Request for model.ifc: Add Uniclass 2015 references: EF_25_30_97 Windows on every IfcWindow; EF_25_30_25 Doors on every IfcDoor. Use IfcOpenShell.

First a look at what the model holds.

```python
import ifcopenshell

model = ifcopenshell.open("model.ifc")
print(model.schema)
print("classifications:", [c.Name for c in model.by_type("IfcClassification")])
for ifc_class in ("IfcDoor", "IfcRoof", "IfcStair", "IfcWall", "IfcWindow"):
    print(ifc_class, len(model.by_type(ifc_class)))
```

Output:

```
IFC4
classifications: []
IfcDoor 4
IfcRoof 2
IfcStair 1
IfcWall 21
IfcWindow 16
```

```python
import ifcopenshell
import ifcopenshell.api.classification

model = ifcopenshell.open("model.ifc")

system = ifcopenshell.api.classification.add_classification(model, classification="Uniclass 2015")

codes = {
    "IfcWindow": ("EF_25_30_97", "Windows"),
    "IfcDoor": ("EF_25_30_25", "Doors"),
}
for ifc_class, (code, name) in codes.items():
    products = model.by_type(ifc_class)
    ifcopenshell.api.classification.add_reference(
        model, products=products, classification=system, identification=code, name=name
    )
    print(code, len(products))

model.write("model_edited.ifc")
```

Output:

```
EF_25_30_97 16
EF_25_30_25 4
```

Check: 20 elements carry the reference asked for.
